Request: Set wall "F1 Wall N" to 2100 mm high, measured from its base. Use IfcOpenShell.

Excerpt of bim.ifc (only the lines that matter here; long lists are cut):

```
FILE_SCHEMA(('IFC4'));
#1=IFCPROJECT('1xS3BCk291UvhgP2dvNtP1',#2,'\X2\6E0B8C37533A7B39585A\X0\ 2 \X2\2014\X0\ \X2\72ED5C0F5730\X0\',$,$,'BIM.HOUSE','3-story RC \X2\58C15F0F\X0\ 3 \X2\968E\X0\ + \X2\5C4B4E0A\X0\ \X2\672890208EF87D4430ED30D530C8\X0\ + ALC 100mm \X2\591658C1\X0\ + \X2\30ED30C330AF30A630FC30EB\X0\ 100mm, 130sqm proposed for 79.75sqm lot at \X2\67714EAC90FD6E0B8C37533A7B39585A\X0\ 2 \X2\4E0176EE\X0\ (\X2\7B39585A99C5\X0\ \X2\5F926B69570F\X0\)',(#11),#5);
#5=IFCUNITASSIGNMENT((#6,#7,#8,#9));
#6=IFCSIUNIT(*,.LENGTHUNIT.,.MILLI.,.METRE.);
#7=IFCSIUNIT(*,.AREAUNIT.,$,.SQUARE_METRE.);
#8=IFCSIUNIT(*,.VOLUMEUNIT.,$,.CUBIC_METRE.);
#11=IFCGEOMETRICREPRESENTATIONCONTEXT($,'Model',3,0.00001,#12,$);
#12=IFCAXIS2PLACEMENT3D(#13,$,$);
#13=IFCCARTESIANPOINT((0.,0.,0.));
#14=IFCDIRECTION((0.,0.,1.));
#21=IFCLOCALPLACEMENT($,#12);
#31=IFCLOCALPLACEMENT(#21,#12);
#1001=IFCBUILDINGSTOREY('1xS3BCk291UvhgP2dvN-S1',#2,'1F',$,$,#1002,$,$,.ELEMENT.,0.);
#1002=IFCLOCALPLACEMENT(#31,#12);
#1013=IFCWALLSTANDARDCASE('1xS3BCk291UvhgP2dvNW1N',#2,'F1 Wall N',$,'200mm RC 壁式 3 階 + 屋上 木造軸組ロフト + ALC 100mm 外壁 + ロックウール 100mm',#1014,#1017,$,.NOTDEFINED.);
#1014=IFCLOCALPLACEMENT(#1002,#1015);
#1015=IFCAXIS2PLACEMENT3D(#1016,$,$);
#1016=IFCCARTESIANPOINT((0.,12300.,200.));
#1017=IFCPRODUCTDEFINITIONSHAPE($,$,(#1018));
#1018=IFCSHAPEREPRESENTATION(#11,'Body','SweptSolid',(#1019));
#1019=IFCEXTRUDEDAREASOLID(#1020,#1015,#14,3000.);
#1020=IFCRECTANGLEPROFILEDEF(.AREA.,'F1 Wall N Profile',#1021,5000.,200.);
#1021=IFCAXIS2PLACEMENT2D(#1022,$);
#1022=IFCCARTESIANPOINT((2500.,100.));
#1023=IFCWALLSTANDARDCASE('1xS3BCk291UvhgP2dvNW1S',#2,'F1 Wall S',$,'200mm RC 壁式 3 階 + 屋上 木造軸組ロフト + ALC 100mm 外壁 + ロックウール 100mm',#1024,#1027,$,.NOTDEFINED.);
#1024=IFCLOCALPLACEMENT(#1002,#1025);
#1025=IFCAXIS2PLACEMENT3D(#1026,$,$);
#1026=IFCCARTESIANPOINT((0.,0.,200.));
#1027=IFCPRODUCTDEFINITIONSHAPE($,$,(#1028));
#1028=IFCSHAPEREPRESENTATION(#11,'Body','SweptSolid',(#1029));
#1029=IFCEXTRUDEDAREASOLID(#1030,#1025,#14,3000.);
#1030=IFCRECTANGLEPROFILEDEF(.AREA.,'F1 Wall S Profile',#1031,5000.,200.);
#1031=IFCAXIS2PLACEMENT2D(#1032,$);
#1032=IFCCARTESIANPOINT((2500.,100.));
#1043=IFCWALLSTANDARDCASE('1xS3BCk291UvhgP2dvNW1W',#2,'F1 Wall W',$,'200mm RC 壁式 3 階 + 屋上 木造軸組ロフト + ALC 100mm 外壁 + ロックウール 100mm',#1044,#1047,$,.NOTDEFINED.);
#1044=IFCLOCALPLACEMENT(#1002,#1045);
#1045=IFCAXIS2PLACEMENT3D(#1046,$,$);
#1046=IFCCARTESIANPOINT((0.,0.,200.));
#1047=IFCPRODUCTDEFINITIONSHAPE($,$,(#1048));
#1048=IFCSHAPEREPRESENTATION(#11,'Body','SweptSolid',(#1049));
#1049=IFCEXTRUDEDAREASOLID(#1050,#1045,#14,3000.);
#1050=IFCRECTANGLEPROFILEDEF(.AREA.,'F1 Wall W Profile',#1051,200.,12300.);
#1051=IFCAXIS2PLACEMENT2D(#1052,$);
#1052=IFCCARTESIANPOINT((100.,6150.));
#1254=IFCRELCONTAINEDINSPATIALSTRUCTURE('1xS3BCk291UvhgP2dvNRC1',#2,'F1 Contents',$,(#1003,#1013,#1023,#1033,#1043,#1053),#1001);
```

```python
import ifcopenshell
import ifcopenshell.geom
import ifcopenshell.util.shape
import ifcopenshell.util.unit

model = ifcopenshell.open("bim.ifc")
unit_scale = ifcopenshell.util.unit.calculate_unit_scale(model)
settings = ifcopenshell.geom.settings()


def volume(element):
    """Net volume in cubic metres, openings subtracted."""
    shape = ifcopenshell.geom.create_shape(settings, element)
    return ifcopenshell.util.shape.get_volume(shape.geometry)


wall = model.by_id(1013)
before = volume(wall)

body = next(r for r in wall.Representation.Representations if r.RepresentationIdentifier == "Body")
solid = body.Items[0]
old_height = solid.Depth
solid.Depth = 2.1 / unit_scale
after = volume(wall)

print(f"height {old_height:g} -> {solid.Depth:g}, volume {before:.3f} -> {after:.3f} m3")

model.write("bim_edited.ifc")
```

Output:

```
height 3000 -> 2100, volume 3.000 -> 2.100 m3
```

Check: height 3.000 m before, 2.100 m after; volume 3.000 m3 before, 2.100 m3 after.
